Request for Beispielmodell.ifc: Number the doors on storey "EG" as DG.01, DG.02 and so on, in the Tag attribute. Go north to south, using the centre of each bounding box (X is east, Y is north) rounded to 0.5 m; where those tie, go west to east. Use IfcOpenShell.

First a look at what the model holds.

```python
import ifcopenshell
import ifcopenshell.util.element
import ifcopenshell.util.placement

model = ifcopenshell.open("Beispielmodell.ifc")
print(model.schema)
storey = next(s for s in model.by_type("IfcBuildingStorey") if s.Name == "EG")
doors = [e for e in ifcopenshell.util.element.get_decomposition(storey) if e.is_a("IfcDoor")]
for e in sorted(doors, key=lambda e: e.id()):
    origin = ifcopenshell.util.placement.get_local_placement(e.ObjectPlacement)[:3, 3]
    print(e.id(), e.Tag, e.Name, origin.round(2) + 0.0, sep=" | ")
```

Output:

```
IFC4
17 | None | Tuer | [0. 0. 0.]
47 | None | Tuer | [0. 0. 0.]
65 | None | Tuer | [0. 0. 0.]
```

```python
import ifcopenshell
import ifcopenshell.geom
import ifcopenshell.util.element
import ifcopenshell.util.shape

model = ifcopenshell.open("Beispielmodell.ifc")
settings = ifcopenshell.geom.settings()
settings.set("use-world-coords", True)


def centre(element):
    shape = ifcopenshell.geom.create_shape(settings, element)
    return ifcopenshell.util.shape.get_bbox_centroid(shape.geometry)


storey = next(s for s in model.by_type("IfcBuildingStorey") if s.Name == "EG")
doors = [e for e in ifcopenshell.util.element.get_decomposition(storey) if e.is_a("IfcDoor")]

# Insertion points can sit at a corner or the storey origin, so sort by the geometry (in metres).
centres = {e: centre(e) for e in doors}
doors.sort(key=lambda e: (-round(centres[e][1] / 0.5), centres[e][0]))

for i, e in enumerate(doors, start=1):
    number = f"DG.{i:02d}"
    e.Tag = number
    print(e.id(), number)

model.write("Beispielmodell-out.ifc")
```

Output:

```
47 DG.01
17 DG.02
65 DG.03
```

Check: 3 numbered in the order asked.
